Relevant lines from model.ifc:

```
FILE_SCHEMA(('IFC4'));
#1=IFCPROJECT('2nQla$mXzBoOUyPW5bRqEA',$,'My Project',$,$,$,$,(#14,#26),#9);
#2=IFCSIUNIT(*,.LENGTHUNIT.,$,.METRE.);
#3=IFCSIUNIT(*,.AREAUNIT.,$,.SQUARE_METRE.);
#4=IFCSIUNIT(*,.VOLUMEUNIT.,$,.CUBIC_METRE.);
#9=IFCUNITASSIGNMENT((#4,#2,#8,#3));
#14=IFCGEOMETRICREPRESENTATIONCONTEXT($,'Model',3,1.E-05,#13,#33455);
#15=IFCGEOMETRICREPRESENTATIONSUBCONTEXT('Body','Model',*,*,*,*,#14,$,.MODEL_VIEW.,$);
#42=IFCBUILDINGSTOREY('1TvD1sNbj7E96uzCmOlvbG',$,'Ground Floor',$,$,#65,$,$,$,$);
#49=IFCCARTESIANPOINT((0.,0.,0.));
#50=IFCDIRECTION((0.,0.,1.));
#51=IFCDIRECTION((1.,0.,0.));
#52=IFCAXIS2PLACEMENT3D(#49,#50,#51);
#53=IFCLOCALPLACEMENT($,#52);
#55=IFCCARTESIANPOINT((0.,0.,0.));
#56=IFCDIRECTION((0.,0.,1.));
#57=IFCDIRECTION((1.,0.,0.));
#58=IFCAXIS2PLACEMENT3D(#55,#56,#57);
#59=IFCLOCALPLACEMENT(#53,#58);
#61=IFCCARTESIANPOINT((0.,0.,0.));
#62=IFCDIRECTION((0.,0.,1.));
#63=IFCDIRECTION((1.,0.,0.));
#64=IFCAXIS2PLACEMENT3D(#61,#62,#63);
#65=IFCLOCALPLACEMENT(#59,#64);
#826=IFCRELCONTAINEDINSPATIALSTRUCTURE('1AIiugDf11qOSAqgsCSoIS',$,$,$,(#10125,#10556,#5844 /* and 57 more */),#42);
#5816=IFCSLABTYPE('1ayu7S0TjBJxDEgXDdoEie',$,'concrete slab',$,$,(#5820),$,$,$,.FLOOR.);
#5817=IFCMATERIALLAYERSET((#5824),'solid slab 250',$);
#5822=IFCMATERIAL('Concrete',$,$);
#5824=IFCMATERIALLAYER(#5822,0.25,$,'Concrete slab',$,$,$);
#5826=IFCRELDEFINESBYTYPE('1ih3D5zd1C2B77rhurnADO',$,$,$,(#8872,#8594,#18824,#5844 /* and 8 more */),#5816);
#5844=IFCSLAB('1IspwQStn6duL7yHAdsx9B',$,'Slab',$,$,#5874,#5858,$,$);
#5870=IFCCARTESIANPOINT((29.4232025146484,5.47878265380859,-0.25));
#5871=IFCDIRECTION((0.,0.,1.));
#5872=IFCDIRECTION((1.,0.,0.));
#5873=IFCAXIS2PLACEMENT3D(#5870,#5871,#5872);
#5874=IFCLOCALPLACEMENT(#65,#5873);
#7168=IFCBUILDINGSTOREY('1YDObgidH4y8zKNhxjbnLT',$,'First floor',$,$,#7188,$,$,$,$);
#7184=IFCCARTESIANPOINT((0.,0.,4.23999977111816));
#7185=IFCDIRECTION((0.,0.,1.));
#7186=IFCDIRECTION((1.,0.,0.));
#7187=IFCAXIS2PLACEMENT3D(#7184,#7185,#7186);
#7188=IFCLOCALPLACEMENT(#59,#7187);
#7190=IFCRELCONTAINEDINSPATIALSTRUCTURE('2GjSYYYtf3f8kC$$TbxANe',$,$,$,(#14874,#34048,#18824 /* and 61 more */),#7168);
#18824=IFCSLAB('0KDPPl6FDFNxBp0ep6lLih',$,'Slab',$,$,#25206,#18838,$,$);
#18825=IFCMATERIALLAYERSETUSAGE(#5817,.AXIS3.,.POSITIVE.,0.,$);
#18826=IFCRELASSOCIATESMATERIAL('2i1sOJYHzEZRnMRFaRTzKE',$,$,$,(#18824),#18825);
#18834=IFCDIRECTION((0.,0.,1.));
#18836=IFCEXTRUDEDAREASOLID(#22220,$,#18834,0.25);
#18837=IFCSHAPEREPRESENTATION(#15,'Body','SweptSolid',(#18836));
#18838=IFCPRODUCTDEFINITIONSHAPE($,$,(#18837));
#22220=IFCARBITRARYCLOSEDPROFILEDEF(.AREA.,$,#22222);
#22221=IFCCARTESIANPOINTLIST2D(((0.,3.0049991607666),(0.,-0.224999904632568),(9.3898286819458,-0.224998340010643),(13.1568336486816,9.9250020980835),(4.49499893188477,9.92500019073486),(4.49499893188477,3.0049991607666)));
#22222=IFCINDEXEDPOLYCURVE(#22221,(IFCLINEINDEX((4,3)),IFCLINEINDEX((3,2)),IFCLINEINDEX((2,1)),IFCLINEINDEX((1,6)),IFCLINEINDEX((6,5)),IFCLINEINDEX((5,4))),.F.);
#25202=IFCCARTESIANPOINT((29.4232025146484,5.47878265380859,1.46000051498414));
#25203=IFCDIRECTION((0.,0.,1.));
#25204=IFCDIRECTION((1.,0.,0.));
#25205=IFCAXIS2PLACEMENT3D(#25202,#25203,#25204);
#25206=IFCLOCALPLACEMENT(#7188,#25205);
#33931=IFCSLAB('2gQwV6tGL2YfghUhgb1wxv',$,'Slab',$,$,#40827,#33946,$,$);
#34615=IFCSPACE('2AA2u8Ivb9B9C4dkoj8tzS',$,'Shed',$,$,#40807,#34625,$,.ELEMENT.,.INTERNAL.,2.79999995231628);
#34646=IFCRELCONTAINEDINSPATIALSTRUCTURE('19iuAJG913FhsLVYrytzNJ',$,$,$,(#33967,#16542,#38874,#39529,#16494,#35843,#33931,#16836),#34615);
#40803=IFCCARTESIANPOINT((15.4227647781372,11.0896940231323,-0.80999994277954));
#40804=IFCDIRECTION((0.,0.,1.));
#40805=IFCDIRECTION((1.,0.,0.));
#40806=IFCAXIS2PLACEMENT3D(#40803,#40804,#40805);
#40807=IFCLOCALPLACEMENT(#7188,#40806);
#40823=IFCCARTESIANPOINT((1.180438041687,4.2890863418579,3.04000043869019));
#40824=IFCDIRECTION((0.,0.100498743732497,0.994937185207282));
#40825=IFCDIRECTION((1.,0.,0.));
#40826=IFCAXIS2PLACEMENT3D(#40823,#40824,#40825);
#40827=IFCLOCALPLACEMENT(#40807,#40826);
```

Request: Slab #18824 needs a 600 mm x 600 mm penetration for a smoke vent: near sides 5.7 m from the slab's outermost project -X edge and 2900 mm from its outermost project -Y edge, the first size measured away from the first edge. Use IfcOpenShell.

```python
import numpy as np
import ifcopenshell
import ifcopenshell.api.feature
import ifcopenshell.api.geometry
import ifcopenshell.api.root
import ifcopenshell.geom
import ifcopenshell.util.placement
import ifcopenshell.util.representation
import ifcopenshell.util.shape
import ifcopenshell.util.unit

model = ifcopenshell.open("model.ifc")
unit_scale = ifcopenshell.util.unit.calculate_unit_scale(model)
settings = ifcopenshell.geom.settings()


def volume(element):
    """Net volume in cubic metres, openings subtracted."""
    shape = ifcopenshell.geom.create_shape(settings, element)
    return ifcopenshell.util.shape.get_volume(shape.geometry)


slab = model.by_guid("0KDPPl6FDFNxBp0ep6lLih")
before = volume(slab)

# Extent in the slab's own axes, in metres. The edges named are its -X and -Y sides.
slab_shape = ifcopenshell.geom.create_shape(settings, slab)
vertices = ifcopenshell.util.shape.get_vertices(slab_shape.geometry)
x_min, y_min, bottom = vertices.min(axis=0)
top = vertices[:, 2].max()

opening = ifcopenshell.api.root.create_entity(model, ifc_class="IfcOpeningElement", name="Smoke vent opening", predefined_type="OPENING")
context = ifcopenshell.util.representation.get_context(model, "Model", "Body", "MODEL_VIEW")
width, depth = 0.6, 0.6
outline = [(0.0, 0.0), (width, 0.0), (width, depth), (0.0, depth), (0.0, 0.0)]
# Overshoot both faces by 50 mm so the cut is clean.
shape = ifcopenshell.api.geometry.add_slab_representation(
    model, context=context, depth=top - bottom + 0.1, polyline=outline
)
ifcopenshell.api.geometry.assign_representation(model, product=opening, representation=shape)

matrix = ifcopenshell.util.placement.get_local_placement(slab.ObjectPlacement)
matrix[:, 3] = matrix @ np.append(np.array([x_min + 5.7, y_min + 2.9, bottom - 0.05]) / unit_scale, 1.0)
ifcopenshell.api.geometry.edit_object_placement(model, product=opening, matrix=matrix, is_si=False)
ifcopenshell.api.feature.add_feature(model, feature=opening, element=slab)

after = volume(slab)

print(f"slab volume {before:.3f} -> {after:.3f} m3")

model.write("model-out.ifc")
```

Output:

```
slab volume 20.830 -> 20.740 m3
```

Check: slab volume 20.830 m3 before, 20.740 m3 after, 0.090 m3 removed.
